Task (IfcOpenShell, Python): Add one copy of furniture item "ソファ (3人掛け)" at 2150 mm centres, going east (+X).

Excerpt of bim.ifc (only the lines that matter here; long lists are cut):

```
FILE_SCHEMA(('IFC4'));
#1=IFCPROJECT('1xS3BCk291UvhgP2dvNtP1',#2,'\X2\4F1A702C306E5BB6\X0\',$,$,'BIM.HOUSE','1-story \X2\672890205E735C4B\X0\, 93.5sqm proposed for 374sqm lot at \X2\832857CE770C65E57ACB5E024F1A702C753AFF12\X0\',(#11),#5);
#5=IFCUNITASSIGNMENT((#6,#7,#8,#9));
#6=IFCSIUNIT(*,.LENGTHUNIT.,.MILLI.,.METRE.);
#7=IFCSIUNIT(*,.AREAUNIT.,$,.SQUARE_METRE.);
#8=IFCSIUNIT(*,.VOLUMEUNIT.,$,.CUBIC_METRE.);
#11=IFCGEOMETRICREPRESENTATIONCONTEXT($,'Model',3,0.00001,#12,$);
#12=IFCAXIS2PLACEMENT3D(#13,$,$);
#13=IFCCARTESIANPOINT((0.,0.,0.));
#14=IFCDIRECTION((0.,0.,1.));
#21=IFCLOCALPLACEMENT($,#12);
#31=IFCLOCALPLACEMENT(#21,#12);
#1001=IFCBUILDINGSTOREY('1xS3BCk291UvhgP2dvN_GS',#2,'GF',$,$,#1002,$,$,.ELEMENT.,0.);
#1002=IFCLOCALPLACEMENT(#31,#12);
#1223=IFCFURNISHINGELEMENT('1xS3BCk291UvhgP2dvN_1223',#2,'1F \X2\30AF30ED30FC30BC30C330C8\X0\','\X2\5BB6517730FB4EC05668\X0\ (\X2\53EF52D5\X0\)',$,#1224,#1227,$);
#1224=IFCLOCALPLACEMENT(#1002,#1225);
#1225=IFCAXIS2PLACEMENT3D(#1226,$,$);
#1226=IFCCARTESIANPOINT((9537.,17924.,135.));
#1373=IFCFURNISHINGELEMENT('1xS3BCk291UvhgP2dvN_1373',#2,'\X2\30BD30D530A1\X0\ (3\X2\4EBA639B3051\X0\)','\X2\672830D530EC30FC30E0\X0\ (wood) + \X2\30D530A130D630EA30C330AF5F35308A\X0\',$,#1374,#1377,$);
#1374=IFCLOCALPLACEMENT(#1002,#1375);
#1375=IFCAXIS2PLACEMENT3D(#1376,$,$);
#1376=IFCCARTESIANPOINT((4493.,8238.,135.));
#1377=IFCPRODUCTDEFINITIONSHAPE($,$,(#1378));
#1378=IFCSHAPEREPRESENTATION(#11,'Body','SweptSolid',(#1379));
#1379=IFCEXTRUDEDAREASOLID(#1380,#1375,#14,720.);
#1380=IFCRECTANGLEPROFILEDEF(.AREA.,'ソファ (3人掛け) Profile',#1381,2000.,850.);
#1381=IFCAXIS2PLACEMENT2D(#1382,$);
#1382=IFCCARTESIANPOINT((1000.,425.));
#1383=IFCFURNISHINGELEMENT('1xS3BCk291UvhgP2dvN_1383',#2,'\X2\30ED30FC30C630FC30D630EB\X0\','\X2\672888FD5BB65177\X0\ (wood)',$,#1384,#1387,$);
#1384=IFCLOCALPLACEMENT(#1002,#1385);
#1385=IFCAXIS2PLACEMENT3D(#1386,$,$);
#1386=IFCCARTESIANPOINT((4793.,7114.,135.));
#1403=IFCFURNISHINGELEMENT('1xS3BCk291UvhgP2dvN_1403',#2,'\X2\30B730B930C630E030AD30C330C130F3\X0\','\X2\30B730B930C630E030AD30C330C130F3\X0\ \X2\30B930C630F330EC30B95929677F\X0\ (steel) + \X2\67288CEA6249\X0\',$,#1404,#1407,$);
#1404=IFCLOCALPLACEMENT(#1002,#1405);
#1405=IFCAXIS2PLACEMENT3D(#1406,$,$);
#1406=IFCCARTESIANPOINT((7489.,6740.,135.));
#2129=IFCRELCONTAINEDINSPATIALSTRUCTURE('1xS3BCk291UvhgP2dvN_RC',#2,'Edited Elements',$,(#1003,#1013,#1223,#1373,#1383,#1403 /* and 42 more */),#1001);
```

```python
import numpy as np
import ifcopenshell
import ifcopenshell.api.geometry
import ifcopenshell.api.root
import ifcopenshell.util.element
import ifcopenshell.util.placement
import ifcopenshell.util.unit

model = ifcopenshell.open("bim.ifc")
unit_scale = ifcopenshell.util.unit.calculate_unit_scale(model)


def reuse_history(source, copy):
    """copy_class also copies each property set's owner history, people and application; keep the originals."""
    for rel in copy.IsDefinedBy:
        if rel.is_a("IfcRelDefinesByProperties") and (history := rel.RelatingPropertyDefinition.OwnerHistory):
            rel.RelatingPropertyDefinition.OwnerHistory = source.OwnerHistory
            ifcopenshell.util.element.remove_deep2(model, history)


source = model.by_guid("1xS3BCk291UvhgP2dvN_1373")
base = ifcopenshell.util.placement.get_local_placement(source.ObjectPlacement)
step = np.array([1.0, 0.0, 0.0]) * 2.15 / unit_scale

for i in range(1, 2):
    copy = ifcopenshell.api.root.copy_class(model, product=source)
    copy.Representation = ifcopenshell.util.element.copy_deep(
        model, source.Representation, exclude=["IfcGeometricRepresentationContext", "IfcRepresentationMap"]
    )
    reuse_history(source, copy)
    matrix = base.copy()
    matrix[:3, 3] += i * step
    print("added at", matrix[:3, 3].round(3) + 0.0)
    ifcopenshell.api.geometry.edit_object_placement(model, product=copy, matrix=matrix, is_si=False)

model.write("bim_edited.ifc")
```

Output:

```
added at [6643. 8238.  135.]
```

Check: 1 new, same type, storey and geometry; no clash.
